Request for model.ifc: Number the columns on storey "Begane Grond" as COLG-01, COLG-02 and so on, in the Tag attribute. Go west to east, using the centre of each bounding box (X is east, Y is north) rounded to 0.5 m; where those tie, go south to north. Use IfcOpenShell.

First a look at what the model holds.

```python
import ifcopenshell
import ifcopenshell.util.element
import ifcopenshell.util.placement

model = ifcopenshell.open("model.ifc")
print(model.schema)
storey = next(s for s in model.by_type("IfcBuildingStorey") if s.Name == "Begane Grond")
columns = [e for e in ifcopenshell.util.element.get_decomposition(storey) if e.is_a("IfcColumn")]
for e in sorted(columns, key=lambda e: e.id()):
    origin = ifcopenshell.util.placement.get_local_placement(e.ObjectPlacement)[:3, 3]
    print(e.id(), e.Tag, e.Name, origin.round(2) + 0.0, sep=" | ")
```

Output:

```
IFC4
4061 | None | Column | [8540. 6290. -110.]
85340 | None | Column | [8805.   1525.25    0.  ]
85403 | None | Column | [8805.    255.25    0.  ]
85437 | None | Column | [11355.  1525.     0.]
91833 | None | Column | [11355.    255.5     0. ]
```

```python
import ifcopenshell
import ifcopenshell.geom
import ifcopenshell.util.element
import ifcopenshell.util.shape

model = ifcopenshell.open("model.ifc")
settings = ifcopenshell.geom.settings()
settings.set("use-world-coords", True)


def centre(element):
    shape = ifcopenshell.geom.create_shape(settings, element)
    return ifcopenshell.util.shape.get_bbox_centroid(shape.geometry)


storey = next(s for s in model.by_type("IfcBuildingStorey") if s.Name == "Begane Grond")
columns = [e for e in ifcopenshell.util.element.get_decomposition(storey) if e.is_a("IfcColumn")]

# Insertion points can sit at a corner or the storey origin, so sort by the geometry (in metres).
centres = {e: centre(e) for e in columns}
columns.sort(key=lambda e: (round(centres[e][0] / 0.5), centres[e][1]))

for i, e in enumerate(columns, start=1):
    number = f"COLG-{i:02d}"
    e.Tag = number
    print(e.id(), number)

model.write("model_rev.ifc")
```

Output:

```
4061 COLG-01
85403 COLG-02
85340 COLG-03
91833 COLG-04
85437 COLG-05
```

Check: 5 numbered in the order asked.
